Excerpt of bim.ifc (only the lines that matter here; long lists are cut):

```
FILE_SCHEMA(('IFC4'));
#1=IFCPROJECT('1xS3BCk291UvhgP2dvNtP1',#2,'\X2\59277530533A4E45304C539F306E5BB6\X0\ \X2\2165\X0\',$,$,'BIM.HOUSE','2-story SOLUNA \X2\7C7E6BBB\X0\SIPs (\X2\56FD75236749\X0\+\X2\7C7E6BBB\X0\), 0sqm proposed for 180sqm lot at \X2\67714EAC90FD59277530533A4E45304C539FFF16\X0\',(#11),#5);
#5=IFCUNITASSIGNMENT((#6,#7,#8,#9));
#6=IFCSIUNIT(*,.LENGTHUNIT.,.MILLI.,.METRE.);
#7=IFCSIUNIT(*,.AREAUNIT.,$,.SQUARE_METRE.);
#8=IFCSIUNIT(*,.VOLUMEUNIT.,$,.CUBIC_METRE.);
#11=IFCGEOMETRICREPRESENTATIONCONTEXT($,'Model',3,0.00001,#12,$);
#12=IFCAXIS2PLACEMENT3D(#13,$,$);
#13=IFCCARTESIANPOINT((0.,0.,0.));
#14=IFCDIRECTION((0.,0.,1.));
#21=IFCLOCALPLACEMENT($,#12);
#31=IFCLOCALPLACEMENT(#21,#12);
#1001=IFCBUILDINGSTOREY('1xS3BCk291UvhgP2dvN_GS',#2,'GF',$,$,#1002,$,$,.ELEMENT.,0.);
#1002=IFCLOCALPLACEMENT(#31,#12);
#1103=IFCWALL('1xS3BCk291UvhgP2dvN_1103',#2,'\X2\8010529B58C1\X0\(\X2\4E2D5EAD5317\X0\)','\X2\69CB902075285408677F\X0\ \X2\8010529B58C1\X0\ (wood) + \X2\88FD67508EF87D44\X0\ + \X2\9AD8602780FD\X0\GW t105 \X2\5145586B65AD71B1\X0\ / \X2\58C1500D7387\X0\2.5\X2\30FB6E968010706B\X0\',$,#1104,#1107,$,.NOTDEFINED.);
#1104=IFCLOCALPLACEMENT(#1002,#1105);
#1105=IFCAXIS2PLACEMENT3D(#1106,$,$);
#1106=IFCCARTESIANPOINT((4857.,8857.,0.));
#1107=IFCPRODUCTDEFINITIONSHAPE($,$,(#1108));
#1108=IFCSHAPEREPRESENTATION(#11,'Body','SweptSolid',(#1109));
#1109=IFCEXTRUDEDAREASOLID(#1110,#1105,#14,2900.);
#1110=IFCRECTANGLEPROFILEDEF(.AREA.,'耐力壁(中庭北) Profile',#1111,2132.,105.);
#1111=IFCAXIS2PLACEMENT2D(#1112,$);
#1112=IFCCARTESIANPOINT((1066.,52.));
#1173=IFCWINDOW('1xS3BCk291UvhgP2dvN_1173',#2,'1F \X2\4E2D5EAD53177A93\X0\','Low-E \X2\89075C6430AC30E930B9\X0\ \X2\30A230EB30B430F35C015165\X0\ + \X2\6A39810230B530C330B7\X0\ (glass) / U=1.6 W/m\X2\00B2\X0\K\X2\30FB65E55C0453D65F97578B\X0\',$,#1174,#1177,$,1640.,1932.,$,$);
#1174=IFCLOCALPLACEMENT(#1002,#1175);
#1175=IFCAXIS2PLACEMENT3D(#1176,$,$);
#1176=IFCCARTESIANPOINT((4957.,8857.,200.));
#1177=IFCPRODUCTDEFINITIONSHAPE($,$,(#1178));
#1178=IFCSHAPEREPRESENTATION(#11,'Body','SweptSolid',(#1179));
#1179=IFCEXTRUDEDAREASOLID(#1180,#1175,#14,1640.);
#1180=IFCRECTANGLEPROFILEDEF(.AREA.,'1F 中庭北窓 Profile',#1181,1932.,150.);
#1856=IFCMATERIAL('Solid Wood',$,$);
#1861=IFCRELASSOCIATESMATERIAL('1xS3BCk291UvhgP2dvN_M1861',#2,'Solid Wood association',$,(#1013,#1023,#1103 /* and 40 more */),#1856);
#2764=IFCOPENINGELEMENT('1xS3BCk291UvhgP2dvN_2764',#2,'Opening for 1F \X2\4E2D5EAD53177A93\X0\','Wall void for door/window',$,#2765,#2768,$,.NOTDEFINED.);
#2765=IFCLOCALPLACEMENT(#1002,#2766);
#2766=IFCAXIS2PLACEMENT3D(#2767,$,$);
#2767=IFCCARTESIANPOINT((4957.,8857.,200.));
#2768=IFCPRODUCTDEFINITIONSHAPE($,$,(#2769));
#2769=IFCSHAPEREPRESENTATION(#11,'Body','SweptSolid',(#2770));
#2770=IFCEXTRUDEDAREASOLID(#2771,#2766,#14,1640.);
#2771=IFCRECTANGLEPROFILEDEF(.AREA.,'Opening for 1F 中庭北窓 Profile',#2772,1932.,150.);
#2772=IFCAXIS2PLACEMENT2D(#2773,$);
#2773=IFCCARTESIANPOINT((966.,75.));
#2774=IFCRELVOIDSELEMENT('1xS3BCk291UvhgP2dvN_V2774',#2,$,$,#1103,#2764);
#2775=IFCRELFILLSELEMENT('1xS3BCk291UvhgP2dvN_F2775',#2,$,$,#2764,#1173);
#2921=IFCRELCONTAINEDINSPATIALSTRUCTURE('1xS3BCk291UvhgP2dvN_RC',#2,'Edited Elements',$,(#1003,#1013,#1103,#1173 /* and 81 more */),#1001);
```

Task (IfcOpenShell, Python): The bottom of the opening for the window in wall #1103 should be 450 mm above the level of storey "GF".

```python
import numpy as np
import ifcopenshell
import ifcopenshell.api.geometry
import ifcopenshell.geom
import ifcopenshell.util.element
import ifcopenshell.util.placement
import ifcopenshell.util.shape
import ifcopenshell.util.unit

model = ifcopenshell.open("bim.ifc")
unit_scale = ifcopenshell.util.unit.calculate_unit_scale(model)

window = model.by_id(1173)
opening = window.FillsVoids[0].RelatingOpeningElement
storey = ifcopenshell.util.element.get_container(window, ifc_class="IfcBuildingStorey")
level = ifcopenshell.util.placement.get_local_placement(storey.ObjectPlacement)[2, 3]

# The opening's origin need not be at the sill, so measure its lowest point.
shape = ifcopenshell.geom.create_shape(ifcopenshell.geom.settings(), opening)
bottom = ifcopenshell.util.shape.get_shape_bottom_elevation(shape, shape.geometry) / unit_scale
dz = level + 0.45 / unit_scale - bottom

shift = np.array([0.0, 0.0, dz])
# The window is not placed relative to its opening, so move both.
for product in (opening, window):
    matrix = ifcopenshell.util.placement.get_local_placement(product.ObjectPlacement)
    matrix[:3, 3] += shift
    ifcopenshell.api.geometry.edit_object_placement(model, product=product, matrix=matrix, is_si=False)

print(f"moved by {dz * unit_scale:+.3f} m")

model.write("bim_updated.ifc")
```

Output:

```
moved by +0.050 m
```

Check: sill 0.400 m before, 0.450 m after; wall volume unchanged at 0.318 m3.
